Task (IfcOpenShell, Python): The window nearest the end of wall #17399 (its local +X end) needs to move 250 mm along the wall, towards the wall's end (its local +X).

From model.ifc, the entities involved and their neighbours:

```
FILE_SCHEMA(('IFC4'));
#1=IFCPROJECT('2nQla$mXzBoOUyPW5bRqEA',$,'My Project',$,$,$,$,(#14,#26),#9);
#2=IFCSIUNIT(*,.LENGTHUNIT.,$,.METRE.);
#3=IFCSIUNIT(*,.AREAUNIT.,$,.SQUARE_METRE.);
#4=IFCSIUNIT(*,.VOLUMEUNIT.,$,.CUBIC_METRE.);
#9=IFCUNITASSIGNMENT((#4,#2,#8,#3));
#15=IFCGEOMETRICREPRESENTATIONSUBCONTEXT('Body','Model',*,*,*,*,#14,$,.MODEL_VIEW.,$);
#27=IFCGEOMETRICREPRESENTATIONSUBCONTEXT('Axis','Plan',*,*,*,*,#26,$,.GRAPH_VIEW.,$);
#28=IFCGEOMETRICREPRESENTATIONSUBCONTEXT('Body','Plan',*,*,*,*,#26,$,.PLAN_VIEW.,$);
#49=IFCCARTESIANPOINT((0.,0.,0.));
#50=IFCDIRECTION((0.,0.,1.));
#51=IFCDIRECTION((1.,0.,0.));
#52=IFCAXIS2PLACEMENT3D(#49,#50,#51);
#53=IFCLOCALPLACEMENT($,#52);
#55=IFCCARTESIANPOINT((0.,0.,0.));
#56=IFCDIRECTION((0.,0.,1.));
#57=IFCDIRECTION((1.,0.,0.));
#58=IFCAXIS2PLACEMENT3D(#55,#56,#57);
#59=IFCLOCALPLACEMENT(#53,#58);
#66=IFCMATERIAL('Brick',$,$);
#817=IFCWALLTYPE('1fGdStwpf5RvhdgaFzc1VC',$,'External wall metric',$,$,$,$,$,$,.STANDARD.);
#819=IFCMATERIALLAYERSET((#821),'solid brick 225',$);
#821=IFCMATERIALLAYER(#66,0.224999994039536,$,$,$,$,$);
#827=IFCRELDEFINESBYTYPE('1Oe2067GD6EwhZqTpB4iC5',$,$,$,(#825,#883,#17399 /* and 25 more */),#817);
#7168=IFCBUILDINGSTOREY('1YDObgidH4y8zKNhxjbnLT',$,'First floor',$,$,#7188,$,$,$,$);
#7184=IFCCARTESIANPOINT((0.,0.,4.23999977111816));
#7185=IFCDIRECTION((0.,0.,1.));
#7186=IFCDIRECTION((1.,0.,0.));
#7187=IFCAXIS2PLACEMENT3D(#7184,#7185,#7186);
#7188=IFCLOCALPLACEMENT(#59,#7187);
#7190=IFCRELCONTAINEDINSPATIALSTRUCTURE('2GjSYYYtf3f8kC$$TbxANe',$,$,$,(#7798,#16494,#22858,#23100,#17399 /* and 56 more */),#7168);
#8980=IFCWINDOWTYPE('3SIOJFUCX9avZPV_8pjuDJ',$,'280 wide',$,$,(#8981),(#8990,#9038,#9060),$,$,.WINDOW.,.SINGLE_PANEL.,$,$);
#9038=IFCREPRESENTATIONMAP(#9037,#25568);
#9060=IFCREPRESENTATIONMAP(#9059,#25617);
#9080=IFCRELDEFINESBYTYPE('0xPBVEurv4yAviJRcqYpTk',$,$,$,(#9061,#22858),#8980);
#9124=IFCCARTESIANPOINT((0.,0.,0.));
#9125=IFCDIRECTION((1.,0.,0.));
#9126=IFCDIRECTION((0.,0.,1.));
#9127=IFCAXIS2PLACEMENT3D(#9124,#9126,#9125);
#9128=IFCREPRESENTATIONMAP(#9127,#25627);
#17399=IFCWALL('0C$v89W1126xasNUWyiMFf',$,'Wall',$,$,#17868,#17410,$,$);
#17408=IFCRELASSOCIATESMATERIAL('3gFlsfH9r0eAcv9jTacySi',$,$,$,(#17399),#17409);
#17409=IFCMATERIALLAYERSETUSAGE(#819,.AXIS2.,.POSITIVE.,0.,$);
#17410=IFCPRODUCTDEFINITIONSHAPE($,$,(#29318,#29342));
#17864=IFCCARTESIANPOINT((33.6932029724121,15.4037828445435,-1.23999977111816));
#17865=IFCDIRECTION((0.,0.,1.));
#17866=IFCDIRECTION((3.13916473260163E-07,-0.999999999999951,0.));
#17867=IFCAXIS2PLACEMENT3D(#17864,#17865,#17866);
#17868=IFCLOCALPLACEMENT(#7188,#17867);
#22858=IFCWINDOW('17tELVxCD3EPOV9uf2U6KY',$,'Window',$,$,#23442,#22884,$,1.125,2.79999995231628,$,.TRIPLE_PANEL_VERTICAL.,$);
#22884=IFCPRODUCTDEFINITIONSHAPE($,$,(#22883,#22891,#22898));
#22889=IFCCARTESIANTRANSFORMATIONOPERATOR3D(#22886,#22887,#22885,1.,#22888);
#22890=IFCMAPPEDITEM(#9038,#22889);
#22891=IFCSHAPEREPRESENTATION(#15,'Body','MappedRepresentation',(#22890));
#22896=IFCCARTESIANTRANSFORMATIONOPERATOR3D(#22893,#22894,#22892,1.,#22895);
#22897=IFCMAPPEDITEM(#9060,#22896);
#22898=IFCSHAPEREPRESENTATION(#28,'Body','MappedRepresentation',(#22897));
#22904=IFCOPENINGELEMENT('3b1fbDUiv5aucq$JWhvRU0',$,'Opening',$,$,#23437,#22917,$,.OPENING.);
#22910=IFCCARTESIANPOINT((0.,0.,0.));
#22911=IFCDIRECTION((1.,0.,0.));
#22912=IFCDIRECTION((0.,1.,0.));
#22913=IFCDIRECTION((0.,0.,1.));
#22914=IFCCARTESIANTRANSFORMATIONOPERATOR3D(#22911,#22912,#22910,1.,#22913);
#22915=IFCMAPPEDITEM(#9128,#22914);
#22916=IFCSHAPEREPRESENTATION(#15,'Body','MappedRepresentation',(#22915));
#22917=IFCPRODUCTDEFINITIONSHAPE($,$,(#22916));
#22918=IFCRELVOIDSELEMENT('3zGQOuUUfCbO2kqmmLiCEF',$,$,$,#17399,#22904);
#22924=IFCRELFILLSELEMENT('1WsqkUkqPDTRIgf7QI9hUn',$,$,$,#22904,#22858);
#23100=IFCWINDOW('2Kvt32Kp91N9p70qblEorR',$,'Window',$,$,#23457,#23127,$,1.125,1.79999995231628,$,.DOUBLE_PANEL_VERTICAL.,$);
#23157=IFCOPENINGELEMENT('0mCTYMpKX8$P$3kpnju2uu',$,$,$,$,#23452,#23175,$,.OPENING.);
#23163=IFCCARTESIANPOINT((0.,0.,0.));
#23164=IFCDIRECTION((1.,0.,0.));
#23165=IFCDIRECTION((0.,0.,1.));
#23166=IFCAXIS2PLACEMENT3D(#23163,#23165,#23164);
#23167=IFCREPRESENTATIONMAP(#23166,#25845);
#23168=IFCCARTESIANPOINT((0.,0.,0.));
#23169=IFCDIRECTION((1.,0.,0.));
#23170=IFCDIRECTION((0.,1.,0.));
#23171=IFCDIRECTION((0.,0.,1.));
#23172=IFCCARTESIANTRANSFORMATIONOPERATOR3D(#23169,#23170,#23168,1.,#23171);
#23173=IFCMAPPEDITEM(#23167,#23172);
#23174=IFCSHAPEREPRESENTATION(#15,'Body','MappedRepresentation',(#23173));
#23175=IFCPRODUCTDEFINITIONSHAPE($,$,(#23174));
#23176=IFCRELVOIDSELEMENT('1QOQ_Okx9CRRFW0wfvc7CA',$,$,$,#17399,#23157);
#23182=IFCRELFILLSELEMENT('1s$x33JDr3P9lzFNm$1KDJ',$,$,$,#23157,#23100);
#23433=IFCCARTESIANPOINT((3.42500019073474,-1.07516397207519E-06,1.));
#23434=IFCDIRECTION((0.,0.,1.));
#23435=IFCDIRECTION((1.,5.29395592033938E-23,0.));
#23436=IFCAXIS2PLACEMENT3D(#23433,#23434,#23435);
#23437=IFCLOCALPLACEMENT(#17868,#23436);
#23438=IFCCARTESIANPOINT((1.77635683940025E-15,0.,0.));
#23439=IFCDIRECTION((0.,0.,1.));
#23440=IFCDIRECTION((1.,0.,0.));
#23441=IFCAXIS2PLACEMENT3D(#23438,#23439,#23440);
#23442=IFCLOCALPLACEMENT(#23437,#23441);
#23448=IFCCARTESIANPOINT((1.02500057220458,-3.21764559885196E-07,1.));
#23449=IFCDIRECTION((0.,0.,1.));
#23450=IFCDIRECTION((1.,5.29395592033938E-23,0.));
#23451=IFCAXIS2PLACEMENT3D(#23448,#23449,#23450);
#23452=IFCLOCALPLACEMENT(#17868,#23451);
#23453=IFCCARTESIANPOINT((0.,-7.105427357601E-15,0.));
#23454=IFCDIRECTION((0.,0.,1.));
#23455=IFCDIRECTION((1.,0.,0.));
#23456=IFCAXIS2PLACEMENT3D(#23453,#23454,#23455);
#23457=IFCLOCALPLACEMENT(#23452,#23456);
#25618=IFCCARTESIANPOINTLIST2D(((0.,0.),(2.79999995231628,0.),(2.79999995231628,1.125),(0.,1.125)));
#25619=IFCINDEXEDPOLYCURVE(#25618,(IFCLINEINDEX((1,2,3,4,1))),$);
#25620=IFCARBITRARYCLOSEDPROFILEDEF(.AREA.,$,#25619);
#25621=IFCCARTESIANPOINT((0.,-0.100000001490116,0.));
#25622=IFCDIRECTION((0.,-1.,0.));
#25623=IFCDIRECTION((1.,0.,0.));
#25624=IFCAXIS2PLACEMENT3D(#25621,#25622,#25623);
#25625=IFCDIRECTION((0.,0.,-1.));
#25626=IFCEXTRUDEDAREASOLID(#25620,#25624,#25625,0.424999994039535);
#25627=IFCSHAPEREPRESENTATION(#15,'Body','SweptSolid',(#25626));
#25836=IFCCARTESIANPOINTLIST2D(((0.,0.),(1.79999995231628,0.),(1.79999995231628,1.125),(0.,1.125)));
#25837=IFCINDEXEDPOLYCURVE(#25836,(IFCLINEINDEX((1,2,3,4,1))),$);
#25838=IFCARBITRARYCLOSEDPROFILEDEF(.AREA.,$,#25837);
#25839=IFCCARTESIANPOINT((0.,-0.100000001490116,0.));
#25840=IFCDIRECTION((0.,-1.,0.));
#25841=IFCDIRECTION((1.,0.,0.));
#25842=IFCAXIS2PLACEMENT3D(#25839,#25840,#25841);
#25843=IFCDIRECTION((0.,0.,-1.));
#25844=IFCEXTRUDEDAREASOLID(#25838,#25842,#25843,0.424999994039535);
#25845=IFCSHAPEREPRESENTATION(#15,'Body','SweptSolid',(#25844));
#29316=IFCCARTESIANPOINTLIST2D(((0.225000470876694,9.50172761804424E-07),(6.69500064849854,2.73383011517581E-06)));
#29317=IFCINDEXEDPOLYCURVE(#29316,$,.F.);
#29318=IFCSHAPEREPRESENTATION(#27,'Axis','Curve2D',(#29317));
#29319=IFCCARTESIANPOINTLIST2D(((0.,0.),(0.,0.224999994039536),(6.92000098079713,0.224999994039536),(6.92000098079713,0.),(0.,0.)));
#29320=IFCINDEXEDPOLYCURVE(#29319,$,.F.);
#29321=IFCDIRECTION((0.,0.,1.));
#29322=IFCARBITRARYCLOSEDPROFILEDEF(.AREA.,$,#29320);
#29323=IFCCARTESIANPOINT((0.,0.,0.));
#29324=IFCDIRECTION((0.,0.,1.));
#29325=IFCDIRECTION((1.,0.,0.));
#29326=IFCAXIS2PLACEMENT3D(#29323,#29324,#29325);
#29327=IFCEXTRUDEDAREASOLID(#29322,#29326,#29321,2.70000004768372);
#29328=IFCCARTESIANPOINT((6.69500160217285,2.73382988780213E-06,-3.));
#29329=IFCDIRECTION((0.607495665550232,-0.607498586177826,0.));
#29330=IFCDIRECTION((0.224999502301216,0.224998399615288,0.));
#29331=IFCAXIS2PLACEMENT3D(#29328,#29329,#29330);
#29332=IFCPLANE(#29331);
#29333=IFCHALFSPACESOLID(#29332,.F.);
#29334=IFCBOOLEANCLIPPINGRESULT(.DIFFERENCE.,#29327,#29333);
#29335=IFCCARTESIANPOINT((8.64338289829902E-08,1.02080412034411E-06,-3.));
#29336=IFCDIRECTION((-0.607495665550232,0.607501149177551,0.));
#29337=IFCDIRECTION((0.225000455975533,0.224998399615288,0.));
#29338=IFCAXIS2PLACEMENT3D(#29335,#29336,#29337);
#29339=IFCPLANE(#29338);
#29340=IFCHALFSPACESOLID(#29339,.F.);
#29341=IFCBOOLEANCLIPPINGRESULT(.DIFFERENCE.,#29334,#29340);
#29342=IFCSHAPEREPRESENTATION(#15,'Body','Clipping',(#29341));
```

```python
import ifcopenshell
import ifcopenshell.api.geometry
import ifcopenshell.util.placement
import ifcopenshell.util.unit

model = ifcopenshell.open("model.ifc")
unit_scale = ifcopenshell.util.unit.calculate_unit_scale(model)

window = model.by_guid("17tELVxCD3EPOV9uf2U6KY")
opening = window.FillsVoids[0].RelatingOpeningElement
wall = opening.VoidsElements[0].RelatingBuildingElement

wall_matrix = ifcopenshell.util.placement.get_local_placement(wall.ObjectPlacement)
shift = wall_matrix[:3, 0] * 0.25 / unit_scale
before = ifcopenshell.util.placement.get_local_placement(window.ObjectPlacement)[:3, 3].copy()

# The window is placed relative to its opening, so it follows when the opening moves.
matrix = ifcopenshell.util.placement.get_local_placement(opening.ObjectPlacement)
matrix[:3, 3] += shift
ifcopenshell.api.geometry.edit_object_placement(
    model, product=opening, matrix=matrix, is_si=False, should_transform_children=True
)

after = ifcopenshell.util.placement.get_local_placement(window.ObjectPlacement)[:3, 3]
print("window moved by", (after - before).round(3) + 0.0)

model.write("model_edited.ifc")
```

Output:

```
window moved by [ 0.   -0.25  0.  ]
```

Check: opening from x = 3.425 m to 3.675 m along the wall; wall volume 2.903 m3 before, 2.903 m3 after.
